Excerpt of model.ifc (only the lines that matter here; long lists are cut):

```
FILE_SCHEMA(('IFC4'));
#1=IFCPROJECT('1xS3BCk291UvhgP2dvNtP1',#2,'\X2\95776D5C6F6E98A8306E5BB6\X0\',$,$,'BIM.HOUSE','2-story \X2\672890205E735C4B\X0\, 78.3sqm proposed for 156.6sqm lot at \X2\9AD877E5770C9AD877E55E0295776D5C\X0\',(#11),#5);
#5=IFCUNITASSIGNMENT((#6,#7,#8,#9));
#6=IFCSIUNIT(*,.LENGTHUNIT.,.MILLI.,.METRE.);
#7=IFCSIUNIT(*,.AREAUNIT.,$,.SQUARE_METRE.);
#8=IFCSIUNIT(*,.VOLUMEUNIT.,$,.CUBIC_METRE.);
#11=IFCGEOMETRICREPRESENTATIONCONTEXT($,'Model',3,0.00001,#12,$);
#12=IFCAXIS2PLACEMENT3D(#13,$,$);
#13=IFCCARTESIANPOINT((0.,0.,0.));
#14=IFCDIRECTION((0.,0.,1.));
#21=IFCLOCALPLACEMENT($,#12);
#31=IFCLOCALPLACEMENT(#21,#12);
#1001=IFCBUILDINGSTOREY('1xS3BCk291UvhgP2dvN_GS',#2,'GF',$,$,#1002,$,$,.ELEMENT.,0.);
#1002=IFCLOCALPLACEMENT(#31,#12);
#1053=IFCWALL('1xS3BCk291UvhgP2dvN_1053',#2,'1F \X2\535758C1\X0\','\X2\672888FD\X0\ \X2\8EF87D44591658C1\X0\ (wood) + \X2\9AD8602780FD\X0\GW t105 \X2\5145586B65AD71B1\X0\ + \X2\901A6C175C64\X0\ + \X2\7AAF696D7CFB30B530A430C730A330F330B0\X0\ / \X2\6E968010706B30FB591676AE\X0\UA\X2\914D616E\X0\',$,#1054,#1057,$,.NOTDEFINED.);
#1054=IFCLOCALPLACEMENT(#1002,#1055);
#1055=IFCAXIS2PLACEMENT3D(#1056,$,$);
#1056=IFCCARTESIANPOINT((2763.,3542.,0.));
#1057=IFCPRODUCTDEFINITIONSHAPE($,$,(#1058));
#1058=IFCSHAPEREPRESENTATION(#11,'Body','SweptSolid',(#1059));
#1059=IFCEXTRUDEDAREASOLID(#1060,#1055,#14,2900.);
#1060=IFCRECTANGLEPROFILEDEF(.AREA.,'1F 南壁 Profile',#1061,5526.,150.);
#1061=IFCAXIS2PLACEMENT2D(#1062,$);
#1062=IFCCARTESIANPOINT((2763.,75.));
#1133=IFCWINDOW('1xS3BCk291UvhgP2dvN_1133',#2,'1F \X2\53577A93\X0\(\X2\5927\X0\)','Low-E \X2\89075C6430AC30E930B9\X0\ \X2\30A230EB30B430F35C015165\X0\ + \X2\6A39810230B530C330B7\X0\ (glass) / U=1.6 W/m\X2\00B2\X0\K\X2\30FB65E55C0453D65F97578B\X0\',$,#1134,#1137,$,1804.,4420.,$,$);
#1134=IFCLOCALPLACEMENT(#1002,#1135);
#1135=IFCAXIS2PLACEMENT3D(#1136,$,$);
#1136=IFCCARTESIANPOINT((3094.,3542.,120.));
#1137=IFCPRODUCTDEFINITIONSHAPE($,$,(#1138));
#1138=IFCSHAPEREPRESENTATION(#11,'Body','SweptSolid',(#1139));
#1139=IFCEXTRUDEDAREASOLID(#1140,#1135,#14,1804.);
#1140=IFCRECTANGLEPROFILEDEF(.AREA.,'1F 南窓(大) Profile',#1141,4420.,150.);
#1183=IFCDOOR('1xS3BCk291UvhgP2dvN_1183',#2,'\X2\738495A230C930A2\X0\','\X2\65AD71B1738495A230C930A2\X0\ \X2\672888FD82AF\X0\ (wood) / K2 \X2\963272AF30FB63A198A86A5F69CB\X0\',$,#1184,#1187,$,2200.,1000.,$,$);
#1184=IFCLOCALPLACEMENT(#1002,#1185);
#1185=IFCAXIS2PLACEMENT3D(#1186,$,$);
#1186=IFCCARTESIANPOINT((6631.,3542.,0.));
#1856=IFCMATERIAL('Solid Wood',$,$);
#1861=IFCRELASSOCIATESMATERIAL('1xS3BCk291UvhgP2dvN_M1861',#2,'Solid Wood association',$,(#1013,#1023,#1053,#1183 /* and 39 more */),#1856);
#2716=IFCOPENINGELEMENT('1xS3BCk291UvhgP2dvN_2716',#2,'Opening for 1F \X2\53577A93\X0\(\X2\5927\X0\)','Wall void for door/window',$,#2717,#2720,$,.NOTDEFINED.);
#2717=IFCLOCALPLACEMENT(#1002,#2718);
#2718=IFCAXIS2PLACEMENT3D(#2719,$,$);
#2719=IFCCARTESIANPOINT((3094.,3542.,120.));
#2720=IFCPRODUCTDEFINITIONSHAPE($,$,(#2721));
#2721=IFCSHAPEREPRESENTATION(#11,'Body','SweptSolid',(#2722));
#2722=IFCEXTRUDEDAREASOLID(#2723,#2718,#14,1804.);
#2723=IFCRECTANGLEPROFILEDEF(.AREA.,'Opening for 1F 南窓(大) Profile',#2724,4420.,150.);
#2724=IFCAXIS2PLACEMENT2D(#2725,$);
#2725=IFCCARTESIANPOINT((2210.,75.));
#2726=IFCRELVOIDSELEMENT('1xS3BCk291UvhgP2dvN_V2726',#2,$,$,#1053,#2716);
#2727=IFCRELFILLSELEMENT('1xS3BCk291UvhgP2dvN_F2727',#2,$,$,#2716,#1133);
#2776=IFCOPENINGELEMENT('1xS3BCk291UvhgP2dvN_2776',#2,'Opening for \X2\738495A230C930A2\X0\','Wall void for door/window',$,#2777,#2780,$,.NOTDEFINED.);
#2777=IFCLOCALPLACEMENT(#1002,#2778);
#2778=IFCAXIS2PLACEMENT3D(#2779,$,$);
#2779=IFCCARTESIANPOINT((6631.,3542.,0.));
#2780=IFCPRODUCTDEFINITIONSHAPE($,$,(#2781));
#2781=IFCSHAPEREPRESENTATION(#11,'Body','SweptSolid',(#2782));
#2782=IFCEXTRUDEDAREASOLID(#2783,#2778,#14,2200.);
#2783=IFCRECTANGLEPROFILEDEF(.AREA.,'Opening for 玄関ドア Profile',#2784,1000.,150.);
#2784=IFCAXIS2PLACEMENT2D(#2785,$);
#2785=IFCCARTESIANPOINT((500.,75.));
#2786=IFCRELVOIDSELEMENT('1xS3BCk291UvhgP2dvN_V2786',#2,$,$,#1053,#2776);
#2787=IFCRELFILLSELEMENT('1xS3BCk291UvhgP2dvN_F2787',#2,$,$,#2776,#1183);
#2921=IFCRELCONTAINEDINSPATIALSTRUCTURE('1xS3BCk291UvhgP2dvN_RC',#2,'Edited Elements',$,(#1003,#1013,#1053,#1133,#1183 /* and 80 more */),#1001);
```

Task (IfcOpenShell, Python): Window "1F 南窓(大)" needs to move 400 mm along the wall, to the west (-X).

```python
import ifcopenshell
import ifcopenshell.api.geometry
import ifcopenshell.util.placement

model = ifcopenshell.open("model.ifc")

window = model.by_id(1133)
opening = window.FillsVoids[0].RelatingOpeningElement
wall = opening.VoidsElements[0].RelatingBuildingElement

wall_matrix = ifcopenshell.util.placement.get_local_placement(wall.ObjectPlacement)
shift = wall_matrix[:3, 0] * -400.0
before = ifcopenshell.util.placement.get_local_placement(window.ObjectPlacement)[:3, 3].copy()

# The window is not placed relative to its opening, so move both.
for product in (opening, window):
    matrix = ifcopenshell.util.placement.get_local_placement(product.ObjectPlacement)
    matrix[:3, 3] += shift
    ifcopenshell.api.geometry.edit_object_placement(model, product=product, matrix=matrix, is_si=False)

after = ifcopenshell.util.placement.get_local_placement(window.ObjectPlacement)[:3, 3]
print("window moved by", (after - before).round(3) + 0.0)

model.write("model_v2.ifc")
```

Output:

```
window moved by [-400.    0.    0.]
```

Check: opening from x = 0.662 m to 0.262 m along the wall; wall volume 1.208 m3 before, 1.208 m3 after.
